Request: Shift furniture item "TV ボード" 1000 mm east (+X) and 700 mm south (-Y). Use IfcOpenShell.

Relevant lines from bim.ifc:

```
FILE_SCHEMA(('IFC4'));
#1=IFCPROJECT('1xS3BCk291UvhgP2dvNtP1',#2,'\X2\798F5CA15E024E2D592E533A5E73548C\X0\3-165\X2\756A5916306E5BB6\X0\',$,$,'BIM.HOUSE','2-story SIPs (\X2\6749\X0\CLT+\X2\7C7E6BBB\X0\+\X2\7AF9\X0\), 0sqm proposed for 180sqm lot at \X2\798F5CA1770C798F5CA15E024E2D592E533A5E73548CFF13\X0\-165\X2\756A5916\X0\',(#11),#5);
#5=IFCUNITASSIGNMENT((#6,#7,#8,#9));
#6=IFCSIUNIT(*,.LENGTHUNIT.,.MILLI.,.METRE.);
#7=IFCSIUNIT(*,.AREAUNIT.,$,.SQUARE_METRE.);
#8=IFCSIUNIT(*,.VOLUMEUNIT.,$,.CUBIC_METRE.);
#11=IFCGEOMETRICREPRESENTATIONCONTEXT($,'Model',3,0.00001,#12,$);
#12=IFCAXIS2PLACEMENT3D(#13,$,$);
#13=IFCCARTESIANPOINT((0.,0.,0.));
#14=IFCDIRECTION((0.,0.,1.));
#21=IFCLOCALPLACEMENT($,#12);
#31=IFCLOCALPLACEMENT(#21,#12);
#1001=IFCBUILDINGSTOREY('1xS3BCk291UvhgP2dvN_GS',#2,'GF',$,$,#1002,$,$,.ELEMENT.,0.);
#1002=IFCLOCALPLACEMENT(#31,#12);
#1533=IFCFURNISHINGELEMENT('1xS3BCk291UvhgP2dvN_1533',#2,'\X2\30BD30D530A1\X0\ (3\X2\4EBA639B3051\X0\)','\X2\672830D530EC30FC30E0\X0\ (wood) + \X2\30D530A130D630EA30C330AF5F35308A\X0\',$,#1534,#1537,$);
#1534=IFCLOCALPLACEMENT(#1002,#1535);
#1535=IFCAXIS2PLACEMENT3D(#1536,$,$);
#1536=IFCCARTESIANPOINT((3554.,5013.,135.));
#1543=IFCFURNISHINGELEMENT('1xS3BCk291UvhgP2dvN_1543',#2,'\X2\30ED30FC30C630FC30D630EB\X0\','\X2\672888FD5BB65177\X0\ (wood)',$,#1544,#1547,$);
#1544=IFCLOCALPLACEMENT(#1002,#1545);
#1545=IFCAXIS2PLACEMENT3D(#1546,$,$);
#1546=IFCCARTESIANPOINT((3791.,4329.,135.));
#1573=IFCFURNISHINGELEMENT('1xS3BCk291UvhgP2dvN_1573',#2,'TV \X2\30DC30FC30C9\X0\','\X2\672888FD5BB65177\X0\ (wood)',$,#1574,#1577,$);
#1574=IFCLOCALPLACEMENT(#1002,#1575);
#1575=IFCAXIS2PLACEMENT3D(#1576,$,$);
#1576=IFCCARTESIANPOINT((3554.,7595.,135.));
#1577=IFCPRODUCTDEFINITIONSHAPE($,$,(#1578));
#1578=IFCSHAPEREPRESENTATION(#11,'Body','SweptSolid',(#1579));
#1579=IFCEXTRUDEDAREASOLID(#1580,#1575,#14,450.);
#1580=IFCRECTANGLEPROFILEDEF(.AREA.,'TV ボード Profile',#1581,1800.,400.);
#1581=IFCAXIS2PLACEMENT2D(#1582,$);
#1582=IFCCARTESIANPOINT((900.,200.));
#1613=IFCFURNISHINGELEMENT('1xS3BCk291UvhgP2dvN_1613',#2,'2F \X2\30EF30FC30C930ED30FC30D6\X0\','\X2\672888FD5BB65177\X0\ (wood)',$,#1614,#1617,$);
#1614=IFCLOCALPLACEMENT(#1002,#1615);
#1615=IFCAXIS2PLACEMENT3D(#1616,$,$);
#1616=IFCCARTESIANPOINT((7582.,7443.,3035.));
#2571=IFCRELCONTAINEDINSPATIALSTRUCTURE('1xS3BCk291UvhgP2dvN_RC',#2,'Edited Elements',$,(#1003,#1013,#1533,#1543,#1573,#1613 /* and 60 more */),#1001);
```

```python
import ifcopenshell
import ifcopenshell.api.geometry
import ifcopenshell.util.placement
import ifcopenshell.util.unit

model = ifcopenshell.open("bim.ifc")
unit_scale = ifcopenshell.util.unit.calculate_unit_scale(model)

item = model.by_guid("1xS3BCk291UvhgP2dvN_1573")
matrix = ifcopenshell.util.placement.get_local_placement(item.ObjectPlacement)
matrix[0, 3] += 1 / unit_scale
matrix[1, 3] -= 0.7 / unit_scale
ifcopenshell.api.geometry.edit_object_placement(model, product=item, matrix=matrix, is_si=False)

print(ifcopenshell.util.placement.get_local_placement(item.ObjectPlacement).round(3) + 0.0)

model.write("bim-out.ifc")
```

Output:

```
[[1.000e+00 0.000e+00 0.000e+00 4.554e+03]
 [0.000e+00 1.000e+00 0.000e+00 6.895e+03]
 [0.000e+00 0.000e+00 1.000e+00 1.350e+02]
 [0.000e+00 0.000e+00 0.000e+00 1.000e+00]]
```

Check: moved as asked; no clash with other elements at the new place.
